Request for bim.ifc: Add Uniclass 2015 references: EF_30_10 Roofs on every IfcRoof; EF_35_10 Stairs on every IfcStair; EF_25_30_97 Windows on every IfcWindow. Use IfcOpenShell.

First a look at what the model holds.

```python
import ifcopenshell

model = ifcopenshell.open("bim.ifc")
print(model.schema)
print("classifications:", [c.Name for c in model.by_type("IfcClassification")])
for ifc_class in ("IfcDoor", "IfcRoof", "IfcStair", "IfcWall", "IfcWindow"):
    print(ifc_class, len(model.by_type(ifc_class)))
```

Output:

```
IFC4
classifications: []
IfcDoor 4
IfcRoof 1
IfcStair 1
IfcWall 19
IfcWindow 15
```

```python
import ifcopenshell
import ifcopenshell.api.classification

model = ifcopenshell.open("bim.ifc")

system = ifcopenshell.api.classification.add_classification(model, classification="Uniclass 2015")

codes = {
    "IfcRoof": ("EF_30_10", "Roofs"),
    "IfcStair": ("EF_35_10", "Stairs"),
    "IfcWindow": ("EF_25_30_97", "Windows"),
}
for ifc_class, (code, name) in codes.items():
    products = model.by_type(ifc_class)
    ifcopenshell.api.classification.add_reference(
        model, products=products, classification=system, identification=code, name=name
    )
    print(code, len(products))

model.write("bim-out.ifc")
```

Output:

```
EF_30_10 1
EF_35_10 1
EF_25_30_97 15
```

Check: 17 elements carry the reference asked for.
